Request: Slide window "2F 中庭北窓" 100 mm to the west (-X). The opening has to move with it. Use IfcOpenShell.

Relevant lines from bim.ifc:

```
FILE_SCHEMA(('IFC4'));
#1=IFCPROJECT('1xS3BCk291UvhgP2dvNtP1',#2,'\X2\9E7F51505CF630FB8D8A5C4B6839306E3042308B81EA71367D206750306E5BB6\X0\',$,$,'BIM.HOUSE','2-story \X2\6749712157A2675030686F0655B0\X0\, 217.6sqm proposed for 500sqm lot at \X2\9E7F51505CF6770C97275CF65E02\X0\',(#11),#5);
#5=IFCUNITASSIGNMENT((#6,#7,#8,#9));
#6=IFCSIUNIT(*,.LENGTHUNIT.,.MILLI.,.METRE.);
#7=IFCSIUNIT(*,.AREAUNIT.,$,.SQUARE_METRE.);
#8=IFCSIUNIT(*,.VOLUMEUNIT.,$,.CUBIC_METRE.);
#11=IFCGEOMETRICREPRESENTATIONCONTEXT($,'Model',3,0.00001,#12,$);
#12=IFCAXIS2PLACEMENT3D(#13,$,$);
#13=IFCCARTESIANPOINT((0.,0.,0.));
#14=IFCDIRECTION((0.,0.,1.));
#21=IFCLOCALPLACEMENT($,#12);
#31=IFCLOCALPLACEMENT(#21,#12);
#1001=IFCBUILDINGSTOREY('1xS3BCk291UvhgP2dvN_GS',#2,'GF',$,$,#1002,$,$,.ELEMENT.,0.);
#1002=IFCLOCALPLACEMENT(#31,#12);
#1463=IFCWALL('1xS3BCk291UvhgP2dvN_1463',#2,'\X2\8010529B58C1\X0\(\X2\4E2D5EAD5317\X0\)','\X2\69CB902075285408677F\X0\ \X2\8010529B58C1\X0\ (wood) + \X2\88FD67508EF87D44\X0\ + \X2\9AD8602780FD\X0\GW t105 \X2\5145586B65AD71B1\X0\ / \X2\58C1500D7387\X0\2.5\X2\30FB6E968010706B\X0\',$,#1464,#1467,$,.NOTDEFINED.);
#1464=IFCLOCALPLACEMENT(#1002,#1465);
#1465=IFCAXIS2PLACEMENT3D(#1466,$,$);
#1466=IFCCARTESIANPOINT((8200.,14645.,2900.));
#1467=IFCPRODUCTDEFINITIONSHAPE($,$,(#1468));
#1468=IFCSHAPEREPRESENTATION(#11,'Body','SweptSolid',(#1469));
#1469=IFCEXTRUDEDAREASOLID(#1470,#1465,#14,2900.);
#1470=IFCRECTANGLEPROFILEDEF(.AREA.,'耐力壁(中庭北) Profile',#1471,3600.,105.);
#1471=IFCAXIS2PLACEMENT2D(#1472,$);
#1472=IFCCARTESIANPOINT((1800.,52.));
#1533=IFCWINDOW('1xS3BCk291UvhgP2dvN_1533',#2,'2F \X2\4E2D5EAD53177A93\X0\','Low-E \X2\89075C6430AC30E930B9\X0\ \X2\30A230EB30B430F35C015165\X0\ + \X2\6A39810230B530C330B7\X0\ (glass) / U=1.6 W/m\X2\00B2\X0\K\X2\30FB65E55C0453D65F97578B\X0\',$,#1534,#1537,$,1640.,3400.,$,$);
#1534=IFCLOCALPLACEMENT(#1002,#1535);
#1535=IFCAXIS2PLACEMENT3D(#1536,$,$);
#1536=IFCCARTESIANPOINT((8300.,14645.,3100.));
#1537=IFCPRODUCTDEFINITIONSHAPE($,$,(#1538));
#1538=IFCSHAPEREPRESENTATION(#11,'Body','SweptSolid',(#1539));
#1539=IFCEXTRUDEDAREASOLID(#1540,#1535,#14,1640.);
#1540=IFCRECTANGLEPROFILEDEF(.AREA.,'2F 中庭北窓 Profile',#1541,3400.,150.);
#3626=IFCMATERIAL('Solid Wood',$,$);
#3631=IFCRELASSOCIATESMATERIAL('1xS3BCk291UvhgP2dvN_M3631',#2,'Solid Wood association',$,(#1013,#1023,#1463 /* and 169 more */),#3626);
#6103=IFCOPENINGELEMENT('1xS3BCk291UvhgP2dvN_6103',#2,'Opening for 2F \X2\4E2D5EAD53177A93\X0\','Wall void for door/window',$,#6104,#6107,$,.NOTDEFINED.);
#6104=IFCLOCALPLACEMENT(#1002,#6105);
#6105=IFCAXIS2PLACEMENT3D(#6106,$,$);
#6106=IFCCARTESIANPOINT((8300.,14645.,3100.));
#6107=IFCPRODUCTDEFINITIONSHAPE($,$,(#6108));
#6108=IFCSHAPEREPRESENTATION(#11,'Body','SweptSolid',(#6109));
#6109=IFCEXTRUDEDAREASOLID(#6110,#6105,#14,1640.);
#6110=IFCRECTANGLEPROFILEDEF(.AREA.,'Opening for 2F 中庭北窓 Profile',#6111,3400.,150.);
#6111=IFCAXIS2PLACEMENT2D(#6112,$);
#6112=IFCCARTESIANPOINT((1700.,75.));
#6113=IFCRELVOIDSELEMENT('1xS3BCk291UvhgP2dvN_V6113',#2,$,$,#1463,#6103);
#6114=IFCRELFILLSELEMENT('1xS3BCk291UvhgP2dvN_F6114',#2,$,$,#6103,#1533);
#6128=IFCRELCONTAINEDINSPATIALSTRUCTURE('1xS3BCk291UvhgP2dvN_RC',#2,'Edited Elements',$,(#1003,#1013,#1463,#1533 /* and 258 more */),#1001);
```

```python
import ifcopenshell
import ifcopenshell.api.geometry
import ifcopenshell.util.placement
import ifcopenshell.util.unit

model = ifcopenshell.open("bim.ifc")
unit_scale = ifcopenshell.util.unit.calculate_unit_scale(model)

window = model.by_guid("1xS3BCk291UvhgP2dvN_1533")
opening = window.FillsVoids[0].RelatingOpeningElement
wall = opening.VoidsElements[0].RelatingBuildingElement

wall_matrix = ifcopenshell.util.placement.get_local_placement(wall.ObjectPlacement)
shift = wall_matrix[:3, 0] * -0.1 / unit_scale
before = ifcopenshell.util.placement.get_local_placement(window.ObjectPlacement)[:3, 3].copy()

# The window is not placed relative to its opening, so move both.
for product in (opening, window):
    matrix = ifcopenshell.util.placement.get_local_placement(product.ObjectPlacement)
    matrix[:3, 3] += shift
    ifcopenshell.api.geometry.edit_object_placement(model, product=product, matrix=matrix, is_si=False)

after = ifcopenshell.util.placement.get_local_placement(window.ObjectPlacement)[:3, 3]
print("window moved by", (after - before).round(3) + 0.0)

model.write("bim_updated.ifc")
```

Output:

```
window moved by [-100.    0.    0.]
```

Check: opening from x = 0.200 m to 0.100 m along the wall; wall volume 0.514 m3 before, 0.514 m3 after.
